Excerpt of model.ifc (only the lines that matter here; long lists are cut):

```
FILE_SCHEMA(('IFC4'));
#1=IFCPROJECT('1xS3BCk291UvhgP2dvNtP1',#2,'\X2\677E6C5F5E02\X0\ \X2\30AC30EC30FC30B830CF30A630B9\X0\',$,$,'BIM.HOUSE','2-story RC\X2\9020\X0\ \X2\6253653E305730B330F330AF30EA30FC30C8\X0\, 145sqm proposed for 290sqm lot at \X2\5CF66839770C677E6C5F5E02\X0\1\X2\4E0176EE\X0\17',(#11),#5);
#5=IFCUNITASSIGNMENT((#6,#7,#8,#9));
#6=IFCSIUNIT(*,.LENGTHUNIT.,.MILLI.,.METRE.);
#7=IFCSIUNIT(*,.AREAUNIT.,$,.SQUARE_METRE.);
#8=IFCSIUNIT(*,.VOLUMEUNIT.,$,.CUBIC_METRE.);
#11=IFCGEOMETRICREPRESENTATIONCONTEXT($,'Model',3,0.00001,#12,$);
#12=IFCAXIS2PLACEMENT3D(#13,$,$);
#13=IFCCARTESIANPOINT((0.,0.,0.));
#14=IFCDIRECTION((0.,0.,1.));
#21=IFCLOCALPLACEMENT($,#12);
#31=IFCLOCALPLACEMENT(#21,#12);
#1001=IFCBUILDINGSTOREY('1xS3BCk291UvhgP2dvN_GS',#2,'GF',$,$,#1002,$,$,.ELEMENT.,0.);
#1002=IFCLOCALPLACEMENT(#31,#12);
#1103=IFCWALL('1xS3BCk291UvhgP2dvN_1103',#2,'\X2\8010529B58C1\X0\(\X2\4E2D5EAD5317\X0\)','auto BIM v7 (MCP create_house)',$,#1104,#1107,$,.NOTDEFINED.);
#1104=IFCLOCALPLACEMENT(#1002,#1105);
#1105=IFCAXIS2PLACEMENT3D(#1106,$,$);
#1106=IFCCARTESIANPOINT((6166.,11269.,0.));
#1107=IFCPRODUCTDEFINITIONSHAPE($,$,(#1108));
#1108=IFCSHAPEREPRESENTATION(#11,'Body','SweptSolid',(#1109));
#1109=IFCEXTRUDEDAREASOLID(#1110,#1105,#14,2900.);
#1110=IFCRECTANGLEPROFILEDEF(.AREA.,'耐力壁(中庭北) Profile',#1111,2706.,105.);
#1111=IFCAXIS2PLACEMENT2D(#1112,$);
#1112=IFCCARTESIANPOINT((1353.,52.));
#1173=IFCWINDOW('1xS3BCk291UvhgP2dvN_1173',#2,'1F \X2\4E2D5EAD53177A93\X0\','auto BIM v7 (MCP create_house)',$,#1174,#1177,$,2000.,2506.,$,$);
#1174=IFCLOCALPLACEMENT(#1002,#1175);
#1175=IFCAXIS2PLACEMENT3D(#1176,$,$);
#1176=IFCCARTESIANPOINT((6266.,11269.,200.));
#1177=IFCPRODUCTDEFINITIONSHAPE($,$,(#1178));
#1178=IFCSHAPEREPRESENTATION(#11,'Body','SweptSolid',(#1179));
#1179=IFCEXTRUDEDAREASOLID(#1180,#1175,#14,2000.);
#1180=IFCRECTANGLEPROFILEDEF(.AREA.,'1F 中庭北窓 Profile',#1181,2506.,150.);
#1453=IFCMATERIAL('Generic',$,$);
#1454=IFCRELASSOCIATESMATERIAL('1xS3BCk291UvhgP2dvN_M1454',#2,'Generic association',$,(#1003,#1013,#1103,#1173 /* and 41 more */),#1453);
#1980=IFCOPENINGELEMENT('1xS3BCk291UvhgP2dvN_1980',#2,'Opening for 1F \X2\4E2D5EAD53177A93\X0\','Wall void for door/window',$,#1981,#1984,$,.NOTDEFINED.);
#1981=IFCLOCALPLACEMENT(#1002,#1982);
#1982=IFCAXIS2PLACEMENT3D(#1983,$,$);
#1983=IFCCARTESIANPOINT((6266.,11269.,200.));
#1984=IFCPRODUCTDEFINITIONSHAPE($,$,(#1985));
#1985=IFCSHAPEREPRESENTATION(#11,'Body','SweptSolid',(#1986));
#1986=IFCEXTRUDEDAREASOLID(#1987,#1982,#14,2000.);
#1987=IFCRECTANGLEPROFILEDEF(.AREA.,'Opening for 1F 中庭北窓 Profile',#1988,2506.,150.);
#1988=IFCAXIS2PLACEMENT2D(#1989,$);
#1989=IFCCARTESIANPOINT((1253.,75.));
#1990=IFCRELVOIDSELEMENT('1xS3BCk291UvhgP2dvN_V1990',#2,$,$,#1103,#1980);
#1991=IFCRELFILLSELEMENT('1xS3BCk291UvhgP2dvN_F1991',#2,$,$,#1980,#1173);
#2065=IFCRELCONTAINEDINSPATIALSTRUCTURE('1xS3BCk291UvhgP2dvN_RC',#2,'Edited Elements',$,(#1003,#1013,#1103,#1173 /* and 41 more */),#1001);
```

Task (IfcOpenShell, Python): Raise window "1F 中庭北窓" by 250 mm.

```python
import numpy as np
import ifcopenshell
import ifcopenshell.api.geometry
import ifcopenshell.util.placement
import ifcopenshell.util.unit

model = ifcopenshell.open("model.ifc")
unit_scale = ifcopenshell.util.unit.calculate_unit_scale(model)

window = model.by_guid("1xS3BCk291UvhgP2dvN_1173")
opening = window.FillsVoids[0].RelatingOpeningElement
dz = 0.25 / unit_scale

shift = np.array([0.0, 0.0, dz])
# The window is not placed relative to its opening, so move both.
for product in (opening, window):
    matrix = ifcopenshell.util.placement.get_local_placement(product.ObjectPlacement)
    matrix[:3, 3] += shift
    ifcopenshell.api.geometry.edit_object_placement(model, product=product, matrix=matrix, is_si=False)

print(f"moved by {dz * unit_scale:+.3f} m")

model.write("model_edited.ifc")
```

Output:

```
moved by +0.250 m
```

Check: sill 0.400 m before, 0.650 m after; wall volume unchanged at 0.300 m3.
